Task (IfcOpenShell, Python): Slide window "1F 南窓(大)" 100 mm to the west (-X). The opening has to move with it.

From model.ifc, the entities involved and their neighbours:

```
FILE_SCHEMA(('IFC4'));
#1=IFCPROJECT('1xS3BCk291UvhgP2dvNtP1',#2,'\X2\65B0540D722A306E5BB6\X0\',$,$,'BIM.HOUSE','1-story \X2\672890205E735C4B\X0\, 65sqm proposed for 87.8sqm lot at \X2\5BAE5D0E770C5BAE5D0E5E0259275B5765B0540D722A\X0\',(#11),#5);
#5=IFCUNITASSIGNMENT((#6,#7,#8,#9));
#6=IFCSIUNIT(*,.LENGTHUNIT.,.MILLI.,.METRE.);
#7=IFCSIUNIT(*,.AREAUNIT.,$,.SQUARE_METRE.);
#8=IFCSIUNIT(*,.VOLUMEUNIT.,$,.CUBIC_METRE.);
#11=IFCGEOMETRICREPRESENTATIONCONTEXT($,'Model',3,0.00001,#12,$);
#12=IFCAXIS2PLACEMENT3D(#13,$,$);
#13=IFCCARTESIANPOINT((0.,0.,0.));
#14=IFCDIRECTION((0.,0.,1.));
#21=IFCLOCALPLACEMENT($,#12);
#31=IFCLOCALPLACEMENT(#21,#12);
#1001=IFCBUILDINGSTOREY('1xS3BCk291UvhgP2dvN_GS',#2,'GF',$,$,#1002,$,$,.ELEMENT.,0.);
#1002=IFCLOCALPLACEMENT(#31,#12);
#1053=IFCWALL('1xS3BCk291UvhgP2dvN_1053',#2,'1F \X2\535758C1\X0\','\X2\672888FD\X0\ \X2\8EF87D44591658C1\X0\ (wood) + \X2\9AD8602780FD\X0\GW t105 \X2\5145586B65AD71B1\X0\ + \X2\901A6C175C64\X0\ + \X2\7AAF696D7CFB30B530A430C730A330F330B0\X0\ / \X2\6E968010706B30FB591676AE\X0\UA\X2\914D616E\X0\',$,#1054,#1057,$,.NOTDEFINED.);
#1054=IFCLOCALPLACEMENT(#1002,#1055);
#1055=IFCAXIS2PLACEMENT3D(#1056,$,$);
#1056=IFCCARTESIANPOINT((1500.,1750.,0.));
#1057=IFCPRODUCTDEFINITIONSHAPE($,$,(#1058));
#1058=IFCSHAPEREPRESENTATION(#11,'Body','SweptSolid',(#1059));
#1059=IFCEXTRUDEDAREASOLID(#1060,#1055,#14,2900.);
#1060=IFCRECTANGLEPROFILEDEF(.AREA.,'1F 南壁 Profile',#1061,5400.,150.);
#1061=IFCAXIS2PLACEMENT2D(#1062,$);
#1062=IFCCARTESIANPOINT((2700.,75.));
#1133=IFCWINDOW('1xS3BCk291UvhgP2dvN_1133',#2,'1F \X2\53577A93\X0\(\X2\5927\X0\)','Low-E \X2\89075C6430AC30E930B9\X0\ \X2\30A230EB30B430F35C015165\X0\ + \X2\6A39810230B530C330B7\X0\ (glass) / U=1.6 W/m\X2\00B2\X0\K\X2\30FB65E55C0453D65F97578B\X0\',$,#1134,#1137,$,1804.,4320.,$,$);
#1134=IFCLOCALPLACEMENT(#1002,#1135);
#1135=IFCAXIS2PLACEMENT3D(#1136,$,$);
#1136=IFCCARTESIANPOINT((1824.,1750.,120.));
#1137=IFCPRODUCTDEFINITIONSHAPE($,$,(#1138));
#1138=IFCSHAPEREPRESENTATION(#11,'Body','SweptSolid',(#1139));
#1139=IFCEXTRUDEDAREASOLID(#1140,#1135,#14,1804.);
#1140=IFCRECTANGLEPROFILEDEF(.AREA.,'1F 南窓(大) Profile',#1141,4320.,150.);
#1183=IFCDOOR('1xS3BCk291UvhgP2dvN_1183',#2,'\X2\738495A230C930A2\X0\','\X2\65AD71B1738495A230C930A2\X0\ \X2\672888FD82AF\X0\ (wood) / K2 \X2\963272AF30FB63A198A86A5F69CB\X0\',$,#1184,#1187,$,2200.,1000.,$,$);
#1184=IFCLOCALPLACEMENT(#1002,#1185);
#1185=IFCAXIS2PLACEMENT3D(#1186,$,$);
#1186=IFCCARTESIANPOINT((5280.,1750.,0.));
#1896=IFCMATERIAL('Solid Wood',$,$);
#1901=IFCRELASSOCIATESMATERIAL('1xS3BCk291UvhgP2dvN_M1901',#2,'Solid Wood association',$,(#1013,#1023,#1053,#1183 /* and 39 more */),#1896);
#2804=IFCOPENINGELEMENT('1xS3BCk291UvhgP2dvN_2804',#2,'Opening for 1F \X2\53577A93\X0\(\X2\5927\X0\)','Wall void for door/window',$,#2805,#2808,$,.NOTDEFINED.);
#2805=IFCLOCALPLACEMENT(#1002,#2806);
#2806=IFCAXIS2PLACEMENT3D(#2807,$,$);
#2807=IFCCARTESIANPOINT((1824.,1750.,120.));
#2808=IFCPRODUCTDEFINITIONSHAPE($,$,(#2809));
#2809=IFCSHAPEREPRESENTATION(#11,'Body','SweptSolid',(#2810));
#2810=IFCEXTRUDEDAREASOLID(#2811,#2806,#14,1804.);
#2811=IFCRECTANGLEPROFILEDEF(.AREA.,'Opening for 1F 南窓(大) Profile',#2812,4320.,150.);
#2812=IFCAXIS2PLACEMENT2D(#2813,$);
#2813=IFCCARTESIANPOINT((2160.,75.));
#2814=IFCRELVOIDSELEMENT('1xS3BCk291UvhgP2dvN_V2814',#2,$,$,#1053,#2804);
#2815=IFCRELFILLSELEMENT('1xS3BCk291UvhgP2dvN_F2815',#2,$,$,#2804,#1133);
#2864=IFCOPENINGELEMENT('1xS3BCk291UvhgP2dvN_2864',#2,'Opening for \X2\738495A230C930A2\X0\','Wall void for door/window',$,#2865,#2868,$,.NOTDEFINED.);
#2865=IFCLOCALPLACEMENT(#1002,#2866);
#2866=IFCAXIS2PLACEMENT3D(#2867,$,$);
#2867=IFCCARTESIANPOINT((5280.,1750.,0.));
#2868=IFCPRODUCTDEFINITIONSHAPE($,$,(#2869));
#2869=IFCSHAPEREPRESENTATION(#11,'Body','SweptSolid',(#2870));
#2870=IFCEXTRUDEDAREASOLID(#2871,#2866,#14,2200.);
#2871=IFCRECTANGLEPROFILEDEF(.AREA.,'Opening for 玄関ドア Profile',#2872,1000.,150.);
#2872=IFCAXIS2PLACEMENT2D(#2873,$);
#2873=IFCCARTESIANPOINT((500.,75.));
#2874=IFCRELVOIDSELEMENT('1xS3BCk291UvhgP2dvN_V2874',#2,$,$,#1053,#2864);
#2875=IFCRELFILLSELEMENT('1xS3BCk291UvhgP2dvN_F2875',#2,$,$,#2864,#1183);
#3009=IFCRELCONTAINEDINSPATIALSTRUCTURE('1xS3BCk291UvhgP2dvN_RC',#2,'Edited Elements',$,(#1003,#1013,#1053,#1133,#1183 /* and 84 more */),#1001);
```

```python
import ifcopenshell
import ifcopenshell.api.geometry
import ifcopenshell.util.placement

model = ifcopenshell.open("model.ifc")

window = model.by_guid("1xS3BCk291UvhgP2dvN_1133")
opening = window.FillsVoids[0].RelatingOpeningElement
wall = opening.VoidsElements[0].RelatingBuildingElement

wall_matrix = ifcopenshell.util.placement.get_local_placement(wall.ObjectPlacement)
shift = wall_matrix[:3, 0] * -100.0
before = ifcopenshell.util.placement.get_local_placement(window.ObjectPlacement)[:3, 3].copy()

# The window is not placed relative to its opening, so move both.
for product in (opening, window):
    matrix = ifcopenshell.util.placement.get_local_placement(product.ObjectPlacement)
    matrix[:3, 3] += shift
    ifcopenshell.api.geometry.edit_object_placement(model, product=product, matrix=matrix, is_si=False)

after = ifcopenshell.util.placement.get_local_placement(window.ObjectPlacement)[:3, 3]
print("window moved by", (after - before).round(3) + 0.0)

model.write("model_updated.ifc")
```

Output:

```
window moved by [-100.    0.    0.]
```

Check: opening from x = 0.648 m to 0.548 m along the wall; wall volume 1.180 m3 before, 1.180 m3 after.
